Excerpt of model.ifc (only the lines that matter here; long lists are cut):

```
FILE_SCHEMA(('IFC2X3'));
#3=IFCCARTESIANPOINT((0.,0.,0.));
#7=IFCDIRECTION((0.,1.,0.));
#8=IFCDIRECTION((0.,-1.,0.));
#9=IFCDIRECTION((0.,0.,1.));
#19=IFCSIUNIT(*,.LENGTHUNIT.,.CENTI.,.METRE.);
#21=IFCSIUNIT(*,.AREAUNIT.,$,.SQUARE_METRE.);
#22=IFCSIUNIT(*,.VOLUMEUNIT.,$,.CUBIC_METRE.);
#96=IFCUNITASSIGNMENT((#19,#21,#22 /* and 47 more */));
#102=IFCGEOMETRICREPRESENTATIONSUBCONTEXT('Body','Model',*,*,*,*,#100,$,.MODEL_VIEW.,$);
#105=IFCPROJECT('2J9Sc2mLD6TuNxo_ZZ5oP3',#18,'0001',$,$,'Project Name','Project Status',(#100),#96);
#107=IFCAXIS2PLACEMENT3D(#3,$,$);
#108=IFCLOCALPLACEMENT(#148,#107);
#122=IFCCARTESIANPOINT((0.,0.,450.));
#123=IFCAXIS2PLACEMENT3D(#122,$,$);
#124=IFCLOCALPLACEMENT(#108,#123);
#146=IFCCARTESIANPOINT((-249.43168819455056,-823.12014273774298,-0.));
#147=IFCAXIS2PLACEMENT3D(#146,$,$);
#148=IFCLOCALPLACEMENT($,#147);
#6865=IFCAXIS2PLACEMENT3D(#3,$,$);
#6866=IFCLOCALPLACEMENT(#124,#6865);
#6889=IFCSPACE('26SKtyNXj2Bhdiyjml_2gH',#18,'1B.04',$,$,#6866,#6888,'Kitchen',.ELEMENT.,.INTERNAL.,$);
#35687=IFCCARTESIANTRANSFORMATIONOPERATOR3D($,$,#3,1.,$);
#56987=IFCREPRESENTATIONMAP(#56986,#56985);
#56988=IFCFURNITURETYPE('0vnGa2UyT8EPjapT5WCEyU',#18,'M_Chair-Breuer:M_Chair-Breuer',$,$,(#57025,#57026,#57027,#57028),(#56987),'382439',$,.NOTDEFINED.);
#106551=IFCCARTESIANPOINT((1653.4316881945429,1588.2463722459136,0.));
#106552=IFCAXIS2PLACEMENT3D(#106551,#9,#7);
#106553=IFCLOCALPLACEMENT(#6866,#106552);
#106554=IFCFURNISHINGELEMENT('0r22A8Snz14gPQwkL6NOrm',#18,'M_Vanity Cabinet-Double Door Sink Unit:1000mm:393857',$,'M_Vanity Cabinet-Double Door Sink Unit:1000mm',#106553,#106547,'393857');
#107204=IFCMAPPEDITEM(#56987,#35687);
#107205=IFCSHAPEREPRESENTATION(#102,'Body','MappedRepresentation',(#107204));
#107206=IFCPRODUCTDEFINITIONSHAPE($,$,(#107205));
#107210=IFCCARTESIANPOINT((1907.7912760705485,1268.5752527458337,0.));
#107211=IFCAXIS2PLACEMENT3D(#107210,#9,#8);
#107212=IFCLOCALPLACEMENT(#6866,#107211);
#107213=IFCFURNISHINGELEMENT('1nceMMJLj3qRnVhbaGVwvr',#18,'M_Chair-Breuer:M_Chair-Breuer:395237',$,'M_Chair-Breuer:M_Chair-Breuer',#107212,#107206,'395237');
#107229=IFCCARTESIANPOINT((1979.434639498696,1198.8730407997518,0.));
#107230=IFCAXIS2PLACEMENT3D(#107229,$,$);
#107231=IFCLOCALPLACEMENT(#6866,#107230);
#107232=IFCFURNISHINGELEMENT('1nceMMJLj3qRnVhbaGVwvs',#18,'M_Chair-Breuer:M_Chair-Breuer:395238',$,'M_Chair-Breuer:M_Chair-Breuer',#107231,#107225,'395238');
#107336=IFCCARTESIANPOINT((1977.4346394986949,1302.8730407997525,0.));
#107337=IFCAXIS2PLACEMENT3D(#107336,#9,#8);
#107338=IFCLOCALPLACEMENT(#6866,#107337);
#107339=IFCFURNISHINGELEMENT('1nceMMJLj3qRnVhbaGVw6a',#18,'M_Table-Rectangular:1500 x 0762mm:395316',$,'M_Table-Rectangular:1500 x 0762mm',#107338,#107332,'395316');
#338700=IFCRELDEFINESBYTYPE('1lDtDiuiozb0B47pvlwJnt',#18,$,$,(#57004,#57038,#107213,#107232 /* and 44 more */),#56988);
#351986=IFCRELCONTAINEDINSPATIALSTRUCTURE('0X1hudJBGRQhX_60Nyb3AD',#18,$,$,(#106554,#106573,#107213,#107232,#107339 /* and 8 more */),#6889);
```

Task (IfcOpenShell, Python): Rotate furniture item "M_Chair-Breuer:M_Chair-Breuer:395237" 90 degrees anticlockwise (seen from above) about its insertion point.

```python
import ifcopenshell
import ifcopenshell.api.geometry
import ifcopenshell.util.placement

model = ifcopenshell.open("model.ifc")

item = model.by_guid("1nceMMJLj3qRnVhbaGVwvr")
matrix = ifcopenshell.util.placement.get_local_placement(item.ObjectPlacement)
matrix = matrix @ ifcopenshell.util.placement.rotation(90, "Z")
ifcopenshell.api.geometry.edit_object_placement(model, product=item, matrix=matrix, is_si=False)

print(ifcopenshell.util.placement.get_local_placement(item.ObjectPlacement).round(3) + 0.0)

model.write("model_rev.ifc")
```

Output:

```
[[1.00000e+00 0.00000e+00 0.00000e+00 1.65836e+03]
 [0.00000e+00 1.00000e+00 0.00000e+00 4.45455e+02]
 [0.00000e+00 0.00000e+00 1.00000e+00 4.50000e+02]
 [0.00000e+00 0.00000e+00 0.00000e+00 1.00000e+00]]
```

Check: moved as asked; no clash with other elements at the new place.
